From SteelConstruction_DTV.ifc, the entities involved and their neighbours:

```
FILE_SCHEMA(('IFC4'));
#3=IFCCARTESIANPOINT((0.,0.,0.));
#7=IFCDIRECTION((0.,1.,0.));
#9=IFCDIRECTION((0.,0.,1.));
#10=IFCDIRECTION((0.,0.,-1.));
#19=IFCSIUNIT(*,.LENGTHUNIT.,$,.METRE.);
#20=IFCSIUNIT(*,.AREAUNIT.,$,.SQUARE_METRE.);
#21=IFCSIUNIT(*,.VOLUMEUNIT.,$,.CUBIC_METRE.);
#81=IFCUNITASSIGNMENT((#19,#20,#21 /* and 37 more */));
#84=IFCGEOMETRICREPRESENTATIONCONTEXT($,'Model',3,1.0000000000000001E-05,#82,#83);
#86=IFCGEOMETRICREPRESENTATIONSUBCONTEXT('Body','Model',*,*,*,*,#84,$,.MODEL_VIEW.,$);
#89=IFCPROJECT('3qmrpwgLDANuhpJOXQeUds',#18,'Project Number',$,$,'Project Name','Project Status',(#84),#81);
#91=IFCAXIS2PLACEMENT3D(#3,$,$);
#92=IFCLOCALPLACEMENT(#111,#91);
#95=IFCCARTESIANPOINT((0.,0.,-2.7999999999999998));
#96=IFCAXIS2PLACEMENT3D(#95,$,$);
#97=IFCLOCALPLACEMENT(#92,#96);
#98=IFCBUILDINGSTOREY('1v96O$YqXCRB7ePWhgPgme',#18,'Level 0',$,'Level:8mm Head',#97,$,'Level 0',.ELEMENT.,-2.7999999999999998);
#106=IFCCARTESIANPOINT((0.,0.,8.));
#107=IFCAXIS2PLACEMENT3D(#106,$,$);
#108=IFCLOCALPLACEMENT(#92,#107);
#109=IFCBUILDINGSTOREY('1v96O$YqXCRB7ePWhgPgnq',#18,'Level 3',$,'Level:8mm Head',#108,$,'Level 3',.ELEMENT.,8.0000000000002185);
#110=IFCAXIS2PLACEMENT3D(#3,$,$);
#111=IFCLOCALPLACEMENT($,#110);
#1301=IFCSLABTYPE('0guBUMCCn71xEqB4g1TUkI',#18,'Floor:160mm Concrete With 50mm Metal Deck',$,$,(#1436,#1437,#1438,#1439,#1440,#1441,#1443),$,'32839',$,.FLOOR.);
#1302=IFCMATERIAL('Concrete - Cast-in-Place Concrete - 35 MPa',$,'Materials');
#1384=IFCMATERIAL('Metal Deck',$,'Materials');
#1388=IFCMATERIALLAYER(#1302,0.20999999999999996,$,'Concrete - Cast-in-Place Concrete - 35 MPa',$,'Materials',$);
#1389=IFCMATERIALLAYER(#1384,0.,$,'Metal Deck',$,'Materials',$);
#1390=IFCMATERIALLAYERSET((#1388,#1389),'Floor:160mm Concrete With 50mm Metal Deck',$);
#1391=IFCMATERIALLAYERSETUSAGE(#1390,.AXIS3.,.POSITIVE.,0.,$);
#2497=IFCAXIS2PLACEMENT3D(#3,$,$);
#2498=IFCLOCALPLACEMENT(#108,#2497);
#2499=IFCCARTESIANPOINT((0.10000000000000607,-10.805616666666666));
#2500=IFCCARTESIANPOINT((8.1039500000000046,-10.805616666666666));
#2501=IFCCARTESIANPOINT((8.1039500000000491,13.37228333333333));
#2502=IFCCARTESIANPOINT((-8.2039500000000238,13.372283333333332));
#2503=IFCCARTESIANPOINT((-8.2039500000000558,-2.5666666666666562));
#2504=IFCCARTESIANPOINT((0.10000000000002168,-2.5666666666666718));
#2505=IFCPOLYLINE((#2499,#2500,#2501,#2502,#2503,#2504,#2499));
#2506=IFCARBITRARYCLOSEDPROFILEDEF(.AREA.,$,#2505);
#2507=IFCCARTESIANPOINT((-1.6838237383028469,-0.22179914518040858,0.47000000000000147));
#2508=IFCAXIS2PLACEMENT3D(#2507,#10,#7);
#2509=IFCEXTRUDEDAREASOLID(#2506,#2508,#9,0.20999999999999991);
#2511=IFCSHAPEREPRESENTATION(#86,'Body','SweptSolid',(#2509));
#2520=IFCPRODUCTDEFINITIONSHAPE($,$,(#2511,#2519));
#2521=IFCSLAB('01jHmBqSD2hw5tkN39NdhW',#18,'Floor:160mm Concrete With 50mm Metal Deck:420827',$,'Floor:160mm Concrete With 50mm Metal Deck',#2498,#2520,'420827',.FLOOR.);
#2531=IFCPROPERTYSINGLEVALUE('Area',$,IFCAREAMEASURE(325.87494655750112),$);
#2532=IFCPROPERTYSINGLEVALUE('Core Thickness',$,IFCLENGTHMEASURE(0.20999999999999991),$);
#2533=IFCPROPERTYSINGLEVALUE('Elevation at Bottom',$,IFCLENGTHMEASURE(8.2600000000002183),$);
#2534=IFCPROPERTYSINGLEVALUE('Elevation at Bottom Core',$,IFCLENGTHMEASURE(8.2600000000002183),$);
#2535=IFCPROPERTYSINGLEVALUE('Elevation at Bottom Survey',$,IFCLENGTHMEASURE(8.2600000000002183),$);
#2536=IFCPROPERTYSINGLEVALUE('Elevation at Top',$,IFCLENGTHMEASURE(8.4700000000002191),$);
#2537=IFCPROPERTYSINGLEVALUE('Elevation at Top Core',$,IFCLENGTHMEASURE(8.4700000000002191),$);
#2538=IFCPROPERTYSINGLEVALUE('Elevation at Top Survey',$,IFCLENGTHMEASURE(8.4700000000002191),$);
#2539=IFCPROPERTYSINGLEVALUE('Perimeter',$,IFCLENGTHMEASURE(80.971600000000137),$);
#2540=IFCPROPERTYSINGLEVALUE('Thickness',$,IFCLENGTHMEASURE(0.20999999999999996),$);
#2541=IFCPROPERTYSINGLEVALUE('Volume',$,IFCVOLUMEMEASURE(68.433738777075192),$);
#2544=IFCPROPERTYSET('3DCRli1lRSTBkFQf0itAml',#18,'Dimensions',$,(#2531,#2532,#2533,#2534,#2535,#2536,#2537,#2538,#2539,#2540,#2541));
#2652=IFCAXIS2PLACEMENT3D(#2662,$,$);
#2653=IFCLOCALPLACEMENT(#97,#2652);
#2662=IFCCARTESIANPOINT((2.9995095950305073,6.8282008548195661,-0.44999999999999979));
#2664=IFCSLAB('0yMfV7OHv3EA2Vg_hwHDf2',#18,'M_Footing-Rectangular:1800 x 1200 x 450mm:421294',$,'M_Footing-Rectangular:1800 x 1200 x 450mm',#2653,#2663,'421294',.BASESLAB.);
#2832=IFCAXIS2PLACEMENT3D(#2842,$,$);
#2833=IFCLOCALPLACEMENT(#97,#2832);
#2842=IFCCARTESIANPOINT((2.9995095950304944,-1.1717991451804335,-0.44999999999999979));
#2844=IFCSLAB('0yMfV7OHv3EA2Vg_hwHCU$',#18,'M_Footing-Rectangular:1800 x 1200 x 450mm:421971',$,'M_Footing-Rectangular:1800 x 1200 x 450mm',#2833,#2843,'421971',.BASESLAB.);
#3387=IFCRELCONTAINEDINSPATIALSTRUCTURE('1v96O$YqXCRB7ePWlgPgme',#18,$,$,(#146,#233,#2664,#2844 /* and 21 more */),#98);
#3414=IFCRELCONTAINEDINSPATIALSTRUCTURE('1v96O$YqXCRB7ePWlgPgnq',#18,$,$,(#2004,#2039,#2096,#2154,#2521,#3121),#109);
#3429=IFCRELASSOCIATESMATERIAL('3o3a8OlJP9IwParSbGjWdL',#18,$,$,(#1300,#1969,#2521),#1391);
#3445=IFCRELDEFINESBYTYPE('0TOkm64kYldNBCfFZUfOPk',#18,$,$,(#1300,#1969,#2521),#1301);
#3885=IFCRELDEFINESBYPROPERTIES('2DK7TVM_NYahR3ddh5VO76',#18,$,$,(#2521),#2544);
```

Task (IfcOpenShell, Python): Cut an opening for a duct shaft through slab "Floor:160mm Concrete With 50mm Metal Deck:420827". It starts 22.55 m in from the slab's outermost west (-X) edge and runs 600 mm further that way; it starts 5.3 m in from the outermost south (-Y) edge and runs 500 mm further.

```python
import numpy as np
import ifcopenshell
import ifcopenshell.api.feature
import ifcopenshell.api.geometry
import ifcopenshell.api.pset
import ifcopenshell.api.root
import ifcopenshell.geom
import ifcopenshell.util.element
import ifcopenshell.util.placement
import ifcopenshell.util.representation
import ifcopenshell.util.shape
import ifcopenshell.util.unit

model = ifcopenshell.open("SteelConstruction_DTV.ifc")
unit_scale = ifcopenshell.util.unit.calculate_unit_scale(model)
area_scale = ifcopenshell.util.unit.calculate_unit_scale(model, "AREAUNIT")
volume_scale = ifcopenshell.util.unit.calculate_unit_scale(model, "VOLUMEUNIT")
settings = ifcopenshell.geom.settings()


def volume(element):
    """Net volume in cubic metres, openings subtracted."""
    shape = ifcopenshell.geom.create_shape(settings, element)
    return ifcopenshell.util.shape.get_volume(shape.geometry)


slab = model.by_id(2521)
before = volume(slab)

# Extent in the slab's own axes, in metres. The edges named are its -X and -Y sides.
slab_shape = ifcopenshell.geom.create_shape(settings, slab)
vertices = ifcopenshell.util.shape.get_vertices(slab_shape.geometry)
x_min, y_min, bottom = vertices.min(axis=0)
top = vertices[:, 2].max()

opening = ifcopenshell.api.root.create_entity(model, ifc_class="IfcOpeningElement", name="Duct shaft opening", predefined_type="OPENING")
context = ifcopenshell.util.representation.get_context(model, "Model", "Body", "MODEL_VIEW")
width, depth = 0.6, 0.5
outline = [(0.0, 0.0), (width, 0.0), (width, depth), (0.0, depth), (0.0, 0.0)]
# Overshoot both faces by 50 mm so the cut is clean.
shape = ifcopenshell.api.geometry.add_slab_representation(
    model, context=context, depth=top - bottom + 0.1, polyline=outline
)
ifcopenshell.api.geometry.assign_representation(model, product=opening, representation=shape)

matrix = ifcopenshell.util.placement.get_local_placement(slab.ObjectPlacement)
matrix[:, 3] = matrix @ np.append(np.array([x_min + 22.55, y_min + 5.3, bottom - 0.05]) / unit_scale, 1.0)
ifcopenshell.api.geometry.edit_object_placement(model, product=opening, matrix=matrix, is_si=False)
ifcopenshell.api.feature.add_feature(model, feature=opening, element=slab)

after = volume(slab)

# Update the slab's stored quantities.
pset = model.by_id(ifcopenshell.util.element.get_pset(slab, "Dimensions", should_inherit=False)["id"])
ifcopenshell.api.pset.edit_pset(model, pset=pset, properties={
    "Area": model.create_entity("IfcAreaMeasure", after / (top - bottom) / area_scale),
    "Volume": model.create_entity("IfcVolumeMeasure", after / volume_scale),
})

print(f"slab volume {before:.3f} -> {after:.3f} m3")

model.write("SteelConstruction_DTV_v2.ifc")
```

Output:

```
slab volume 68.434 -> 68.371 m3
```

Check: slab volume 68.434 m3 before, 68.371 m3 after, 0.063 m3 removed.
